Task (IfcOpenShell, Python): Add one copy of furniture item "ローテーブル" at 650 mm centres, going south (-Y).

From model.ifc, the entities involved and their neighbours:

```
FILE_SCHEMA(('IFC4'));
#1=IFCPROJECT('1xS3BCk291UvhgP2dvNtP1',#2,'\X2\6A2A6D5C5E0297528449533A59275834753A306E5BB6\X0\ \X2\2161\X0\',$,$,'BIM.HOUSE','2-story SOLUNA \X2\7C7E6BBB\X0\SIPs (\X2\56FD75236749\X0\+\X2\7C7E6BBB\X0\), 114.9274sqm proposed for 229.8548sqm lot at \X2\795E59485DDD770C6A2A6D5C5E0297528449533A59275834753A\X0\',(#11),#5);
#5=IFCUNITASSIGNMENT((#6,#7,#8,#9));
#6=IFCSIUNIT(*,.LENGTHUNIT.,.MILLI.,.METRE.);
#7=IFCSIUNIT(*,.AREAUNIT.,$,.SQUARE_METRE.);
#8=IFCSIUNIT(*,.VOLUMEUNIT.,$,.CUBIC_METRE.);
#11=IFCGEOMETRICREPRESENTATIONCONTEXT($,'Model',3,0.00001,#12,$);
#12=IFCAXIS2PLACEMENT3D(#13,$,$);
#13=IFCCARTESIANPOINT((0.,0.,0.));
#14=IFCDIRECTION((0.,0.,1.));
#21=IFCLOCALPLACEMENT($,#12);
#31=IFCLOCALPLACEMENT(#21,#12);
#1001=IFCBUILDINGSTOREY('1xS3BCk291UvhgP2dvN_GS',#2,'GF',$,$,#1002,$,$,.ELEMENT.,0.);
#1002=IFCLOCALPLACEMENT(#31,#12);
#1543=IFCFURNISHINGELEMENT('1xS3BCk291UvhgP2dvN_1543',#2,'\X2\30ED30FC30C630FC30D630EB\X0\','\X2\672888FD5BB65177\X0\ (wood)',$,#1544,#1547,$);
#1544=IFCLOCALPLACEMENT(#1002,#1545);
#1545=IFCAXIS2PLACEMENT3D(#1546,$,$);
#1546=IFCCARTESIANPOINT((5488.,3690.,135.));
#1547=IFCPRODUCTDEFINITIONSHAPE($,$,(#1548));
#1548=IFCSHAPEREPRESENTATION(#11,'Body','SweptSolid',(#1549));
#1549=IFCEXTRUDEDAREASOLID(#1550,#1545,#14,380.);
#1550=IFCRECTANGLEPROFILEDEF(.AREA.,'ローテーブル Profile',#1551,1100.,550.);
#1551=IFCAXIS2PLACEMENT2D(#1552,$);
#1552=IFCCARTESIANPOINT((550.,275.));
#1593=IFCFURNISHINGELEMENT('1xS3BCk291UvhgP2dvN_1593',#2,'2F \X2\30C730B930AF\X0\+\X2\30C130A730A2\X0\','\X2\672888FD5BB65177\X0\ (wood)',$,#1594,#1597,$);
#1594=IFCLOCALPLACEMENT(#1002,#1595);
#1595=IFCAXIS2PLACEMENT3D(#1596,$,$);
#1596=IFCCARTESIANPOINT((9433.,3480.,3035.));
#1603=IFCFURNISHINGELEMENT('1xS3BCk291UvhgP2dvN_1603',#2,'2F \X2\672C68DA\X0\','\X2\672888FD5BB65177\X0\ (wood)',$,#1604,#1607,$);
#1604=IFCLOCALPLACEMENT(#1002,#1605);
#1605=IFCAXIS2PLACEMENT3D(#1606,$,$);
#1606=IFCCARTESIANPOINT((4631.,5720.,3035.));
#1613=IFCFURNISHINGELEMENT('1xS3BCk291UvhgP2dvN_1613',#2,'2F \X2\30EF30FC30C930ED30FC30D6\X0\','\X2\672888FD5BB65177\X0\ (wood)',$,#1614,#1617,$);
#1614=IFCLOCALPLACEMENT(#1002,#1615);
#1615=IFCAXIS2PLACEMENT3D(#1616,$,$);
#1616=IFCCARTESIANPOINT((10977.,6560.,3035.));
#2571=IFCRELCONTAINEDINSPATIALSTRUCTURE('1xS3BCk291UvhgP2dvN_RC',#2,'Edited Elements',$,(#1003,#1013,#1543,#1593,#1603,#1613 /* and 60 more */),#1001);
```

```python
import numpy as np
import ifcopenshell
import ifcopenshell.api.geometry
import ifcopenshell.api.root
import ifcopenshell.util.element
import ifcopenshell.util.placement
import ifcopenshell.util.unit

model = ifcopenshell.open("model.ifc")
unit_scale = ifcopenshell.util.unit.calculate_unit_scale(model)


def reuse_history(source, copy):
    """copy_class also copies each property set's owner history, people and application; keep the originals."""
    for rel in copy.IsDefinedBy:
        if rel.is_a("IfcRelDefinesByProperties") and (history := rel.RelatingPropertyDefinition.OwnerHistory):
            rel.RelatingPropertyDefinition.OwnerHistory = source.OwnerHistory
            ifcopenshell.util.element.remove_deep2(model, history)


source = model.by_guid("1xS3BCk291UvhgP2dvN_1543")
base = ifcopenshell.util.placement.get_local_placement(source.ObjectPlacement)
step = np.array([0.0, -1.0, 0.0]) * 0.65 / unit_scale

for i in range(1, 2):
    copy = ifcopenshell.api.root.copy_class(model, product=source)
    copy.Representation = ifcopenshell.util.element.copy_deep(
        model, source.Representation, exclude=["IfcGeometricRepresentationContext", "IfcRepresentationMap"]
    )
    reuse_history(source, copy)
    matrix = base.copy()
    matrix[:3, 3] += i * step
    print("added at", matrix[:3, 3].round(3) + 0.0)
    ifcopenshell.api.geometry.edit_object_placement(model, product=copy, matrix=matrix, is_si=False)

model.write("model_rev.ifc")
```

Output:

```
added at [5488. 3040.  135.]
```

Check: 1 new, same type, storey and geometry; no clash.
